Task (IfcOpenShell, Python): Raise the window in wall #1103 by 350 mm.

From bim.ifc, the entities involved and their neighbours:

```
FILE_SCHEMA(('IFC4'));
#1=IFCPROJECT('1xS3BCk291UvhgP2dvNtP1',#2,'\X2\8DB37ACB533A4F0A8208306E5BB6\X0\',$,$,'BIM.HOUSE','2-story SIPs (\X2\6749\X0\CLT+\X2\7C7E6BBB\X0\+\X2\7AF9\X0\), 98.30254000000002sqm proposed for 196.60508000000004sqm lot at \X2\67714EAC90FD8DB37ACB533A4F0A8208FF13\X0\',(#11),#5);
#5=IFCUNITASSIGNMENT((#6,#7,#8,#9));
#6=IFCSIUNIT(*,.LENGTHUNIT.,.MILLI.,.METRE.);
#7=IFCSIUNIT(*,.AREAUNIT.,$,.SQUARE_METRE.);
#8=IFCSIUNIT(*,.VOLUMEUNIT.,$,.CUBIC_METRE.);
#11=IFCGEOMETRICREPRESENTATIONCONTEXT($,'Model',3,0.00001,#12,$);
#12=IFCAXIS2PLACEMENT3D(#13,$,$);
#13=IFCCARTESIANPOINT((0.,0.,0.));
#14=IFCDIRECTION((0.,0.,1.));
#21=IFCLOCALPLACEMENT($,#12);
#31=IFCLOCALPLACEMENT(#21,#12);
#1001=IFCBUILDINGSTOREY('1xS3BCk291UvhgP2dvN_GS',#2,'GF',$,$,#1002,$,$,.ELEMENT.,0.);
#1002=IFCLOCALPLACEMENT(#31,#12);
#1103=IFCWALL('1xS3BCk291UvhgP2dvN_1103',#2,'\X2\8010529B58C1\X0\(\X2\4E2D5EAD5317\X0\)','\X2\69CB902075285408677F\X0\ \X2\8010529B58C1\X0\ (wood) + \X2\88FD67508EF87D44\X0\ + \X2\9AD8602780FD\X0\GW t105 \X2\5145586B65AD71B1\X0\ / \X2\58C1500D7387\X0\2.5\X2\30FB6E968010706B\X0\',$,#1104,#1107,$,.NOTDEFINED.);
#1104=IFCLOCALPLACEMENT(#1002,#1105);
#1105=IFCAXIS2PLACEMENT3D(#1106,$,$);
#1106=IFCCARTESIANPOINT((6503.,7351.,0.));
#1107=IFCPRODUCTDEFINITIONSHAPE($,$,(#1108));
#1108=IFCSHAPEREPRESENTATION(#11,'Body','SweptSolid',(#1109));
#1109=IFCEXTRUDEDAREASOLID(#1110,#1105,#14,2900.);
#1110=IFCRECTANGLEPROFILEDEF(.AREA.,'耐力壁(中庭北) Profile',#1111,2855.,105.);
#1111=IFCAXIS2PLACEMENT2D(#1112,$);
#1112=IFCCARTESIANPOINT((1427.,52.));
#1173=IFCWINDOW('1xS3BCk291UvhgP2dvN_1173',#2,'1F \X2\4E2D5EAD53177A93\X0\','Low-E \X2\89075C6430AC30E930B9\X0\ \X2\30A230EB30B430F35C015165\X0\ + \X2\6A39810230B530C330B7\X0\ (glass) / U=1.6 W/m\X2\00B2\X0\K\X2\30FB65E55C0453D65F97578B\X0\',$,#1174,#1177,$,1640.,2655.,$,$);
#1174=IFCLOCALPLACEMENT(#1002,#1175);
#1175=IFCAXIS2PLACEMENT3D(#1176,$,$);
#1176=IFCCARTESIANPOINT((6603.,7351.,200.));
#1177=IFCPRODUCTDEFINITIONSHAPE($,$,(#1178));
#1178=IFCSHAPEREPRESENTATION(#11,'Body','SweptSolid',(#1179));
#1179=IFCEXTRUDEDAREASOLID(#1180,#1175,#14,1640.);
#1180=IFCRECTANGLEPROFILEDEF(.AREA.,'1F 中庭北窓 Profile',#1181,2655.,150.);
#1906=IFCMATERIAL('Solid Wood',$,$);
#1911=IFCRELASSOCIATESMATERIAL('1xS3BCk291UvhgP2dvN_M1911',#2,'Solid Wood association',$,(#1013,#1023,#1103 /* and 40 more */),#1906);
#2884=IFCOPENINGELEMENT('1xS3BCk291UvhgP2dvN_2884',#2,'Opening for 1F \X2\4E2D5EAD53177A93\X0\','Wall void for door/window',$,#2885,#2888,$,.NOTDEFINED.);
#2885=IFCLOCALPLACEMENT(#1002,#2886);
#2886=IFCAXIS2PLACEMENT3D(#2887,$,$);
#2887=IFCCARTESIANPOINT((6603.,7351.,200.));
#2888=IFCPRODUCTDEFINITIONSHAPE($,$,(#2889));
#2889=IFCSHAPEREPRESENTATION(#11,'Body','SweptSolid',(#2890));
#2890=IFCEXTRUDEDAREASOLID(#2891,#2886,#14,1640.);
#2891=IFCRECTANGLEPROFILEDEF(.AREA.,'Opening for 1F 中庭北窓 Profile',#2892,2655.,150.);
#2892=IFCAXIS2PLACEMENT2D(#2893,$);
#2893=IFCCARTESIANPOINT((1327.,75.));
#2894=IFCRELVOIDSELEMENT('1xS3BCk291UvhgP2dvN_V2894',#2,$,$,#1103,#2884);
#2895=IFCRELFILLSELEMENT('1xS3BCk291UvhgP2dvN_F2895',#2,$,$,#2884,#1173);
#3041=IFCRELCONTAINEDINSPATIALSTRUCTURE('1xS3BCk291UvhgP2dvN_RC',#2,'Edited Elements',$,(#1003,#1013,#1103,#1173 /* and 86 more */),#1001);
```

```python
import numpy as np
import ifcopenshell
import ifcopenshell.api.geometry
import ifcopenshell.util.placement
import ifcopenshell.util.unit

model = ifcopenshell.open("bim.ifc")
unit_scale = ifcopenshell.util.unit.calculate_unit_scale(model)

window = model.by_id(1173)
opening = window.FillsVoids[0].RelatingOpeningElement
dz = 350.0

shift = np.array([0.0, 0.0, dz])
# The window is not placed relative to its opening, so move both.
for product in (opening, window):
    matrix = ifcopenshell.util.placement.get_local_placement(product.ObjectPlacement)
    matrix[:3, 3] += shift
    ifcopenshell.api.geometry.edit_object_placement(model, product=product, matrix=matrix, is_si=False)

print(f"moved by {dz * unit_scale:+.3f} m")

model.write("bim_rev.ifc")
```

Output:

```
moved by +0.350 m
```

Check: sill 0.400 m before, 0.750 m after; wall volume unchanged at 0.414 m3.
